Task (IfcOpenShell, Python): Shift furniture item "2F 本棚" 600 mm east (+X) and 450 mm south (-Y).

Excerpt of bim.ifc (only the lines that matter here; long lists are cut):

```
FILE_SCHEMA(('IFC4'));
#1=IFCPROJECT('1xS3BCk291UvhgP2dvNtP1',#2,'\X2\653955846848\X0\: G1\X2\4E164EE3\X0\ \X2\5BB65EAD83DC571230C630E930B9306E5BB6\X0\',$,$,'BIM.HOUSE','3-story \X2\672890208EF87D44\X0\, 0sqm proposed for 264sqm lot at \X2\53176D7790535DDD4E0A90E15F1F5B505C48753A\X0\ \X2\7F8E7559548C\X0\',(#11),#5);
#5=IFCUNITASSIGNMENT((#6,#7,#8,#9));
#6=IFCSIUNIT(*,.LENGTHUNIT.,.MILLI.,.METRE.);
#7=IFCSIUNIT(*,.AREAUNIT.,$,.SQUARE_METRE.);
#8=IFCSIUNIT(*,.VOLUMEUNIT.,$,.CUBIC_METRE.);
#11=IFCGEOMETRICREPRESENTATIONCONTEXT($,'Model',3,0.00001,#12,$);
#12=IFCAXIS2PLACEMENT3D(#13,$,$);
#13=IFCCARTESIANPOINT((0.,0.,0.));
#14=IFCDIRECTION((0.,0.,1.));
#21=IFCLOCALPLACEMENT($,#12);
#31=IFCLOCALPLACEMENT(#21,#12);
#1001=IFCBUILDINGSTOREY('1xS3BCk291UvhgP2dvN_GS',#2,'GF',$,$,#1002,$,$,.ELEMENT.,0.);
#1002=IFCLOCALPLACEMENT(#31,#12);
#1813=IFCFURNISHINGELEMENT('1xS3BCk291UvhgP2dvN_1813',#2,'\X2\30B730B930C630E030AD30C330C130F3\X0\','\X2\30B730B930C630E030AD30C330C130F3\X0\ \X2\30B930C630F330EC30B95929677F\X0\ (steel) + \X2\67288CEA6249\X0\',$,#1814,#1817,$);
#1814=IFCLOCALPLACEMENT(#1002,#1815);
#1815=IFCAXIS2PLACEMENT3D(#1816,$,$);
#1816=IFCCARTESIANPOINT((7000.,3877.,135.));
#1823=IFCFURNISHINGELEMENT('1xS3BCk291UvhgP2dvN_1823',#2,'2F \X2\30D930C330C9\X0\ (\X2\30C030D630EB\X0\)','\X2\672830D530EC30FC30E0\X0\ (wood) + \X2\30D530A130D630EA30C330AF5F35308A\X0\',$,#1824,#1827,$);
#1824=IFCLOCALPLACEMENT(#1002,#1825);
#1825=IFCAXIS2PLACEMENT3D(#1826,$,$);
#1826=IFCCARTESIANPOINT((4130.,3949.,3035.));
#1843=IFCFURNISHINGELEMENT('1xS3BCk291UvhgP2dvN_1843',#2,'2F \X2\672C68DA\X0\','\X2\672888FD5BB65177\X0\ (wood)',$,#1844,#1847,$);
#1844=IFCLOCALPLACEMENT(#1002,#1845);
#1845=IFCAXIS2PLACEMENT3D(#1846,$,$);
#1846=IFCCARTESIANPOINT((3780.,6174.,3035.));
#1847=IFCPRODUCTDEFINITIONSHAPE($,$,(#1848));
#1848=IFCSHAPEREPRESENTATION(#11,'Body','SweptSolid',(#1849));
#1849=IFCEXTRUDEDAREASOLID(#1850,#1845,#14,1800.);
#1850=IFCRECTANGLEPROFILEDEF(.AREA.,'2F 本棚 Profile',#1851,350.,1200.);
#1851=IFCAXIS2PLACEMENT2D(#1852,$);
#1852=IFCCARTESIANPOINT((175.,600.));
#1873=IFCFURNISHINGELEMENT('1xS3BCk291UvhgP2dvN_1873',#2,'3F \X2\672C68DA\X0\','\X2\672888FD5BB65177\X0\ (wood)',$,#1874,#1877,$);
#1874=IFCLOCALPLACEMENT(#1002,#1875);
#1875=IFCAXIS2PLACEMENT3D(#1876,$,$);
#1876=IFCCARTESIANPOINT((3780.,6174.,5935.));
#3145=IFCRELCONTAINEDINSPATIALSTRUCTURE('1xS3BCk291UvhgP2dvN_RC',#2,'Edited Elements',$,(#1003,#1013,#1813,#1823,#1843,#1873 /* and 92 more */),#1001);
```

```python
import ifcopenshell
import ifcopenshell.api.geometry
import ifcopenshell.util.placement
import ifcopenshell.util.unit

model = ifcopenshell.open("bim.ifc")
unit_scale = ifcopenshell.util.unit.calculate_unit_scale(model)

item = model.by_guid("1xS3BCk291UvhgP2dvN_1843")
matrix = ifcopenshell.util.placement.get_local_placement(item.ObjectPlacement)
matrix[0, 3] += 0.6 / unit_scale
matrix[1, 3] -= 0.45 / unit_scale
ifcopenshell.api.geometry.edit_object_placement(model, product=item, matrix=matrix, is_si=False)

print(ifcopenshell.util.placement.get_local_placement(item.ObjectPlacement).round(3) + 0.0)

model.write("bim-out.ifc")
```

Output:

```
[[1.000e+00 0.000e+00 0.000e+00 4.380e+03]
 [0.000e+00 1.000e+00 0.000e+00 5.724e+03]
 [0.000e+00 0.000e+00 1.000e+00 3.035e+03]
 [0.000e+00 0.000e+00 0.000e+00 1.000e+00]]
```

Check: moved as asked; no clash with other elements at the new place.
